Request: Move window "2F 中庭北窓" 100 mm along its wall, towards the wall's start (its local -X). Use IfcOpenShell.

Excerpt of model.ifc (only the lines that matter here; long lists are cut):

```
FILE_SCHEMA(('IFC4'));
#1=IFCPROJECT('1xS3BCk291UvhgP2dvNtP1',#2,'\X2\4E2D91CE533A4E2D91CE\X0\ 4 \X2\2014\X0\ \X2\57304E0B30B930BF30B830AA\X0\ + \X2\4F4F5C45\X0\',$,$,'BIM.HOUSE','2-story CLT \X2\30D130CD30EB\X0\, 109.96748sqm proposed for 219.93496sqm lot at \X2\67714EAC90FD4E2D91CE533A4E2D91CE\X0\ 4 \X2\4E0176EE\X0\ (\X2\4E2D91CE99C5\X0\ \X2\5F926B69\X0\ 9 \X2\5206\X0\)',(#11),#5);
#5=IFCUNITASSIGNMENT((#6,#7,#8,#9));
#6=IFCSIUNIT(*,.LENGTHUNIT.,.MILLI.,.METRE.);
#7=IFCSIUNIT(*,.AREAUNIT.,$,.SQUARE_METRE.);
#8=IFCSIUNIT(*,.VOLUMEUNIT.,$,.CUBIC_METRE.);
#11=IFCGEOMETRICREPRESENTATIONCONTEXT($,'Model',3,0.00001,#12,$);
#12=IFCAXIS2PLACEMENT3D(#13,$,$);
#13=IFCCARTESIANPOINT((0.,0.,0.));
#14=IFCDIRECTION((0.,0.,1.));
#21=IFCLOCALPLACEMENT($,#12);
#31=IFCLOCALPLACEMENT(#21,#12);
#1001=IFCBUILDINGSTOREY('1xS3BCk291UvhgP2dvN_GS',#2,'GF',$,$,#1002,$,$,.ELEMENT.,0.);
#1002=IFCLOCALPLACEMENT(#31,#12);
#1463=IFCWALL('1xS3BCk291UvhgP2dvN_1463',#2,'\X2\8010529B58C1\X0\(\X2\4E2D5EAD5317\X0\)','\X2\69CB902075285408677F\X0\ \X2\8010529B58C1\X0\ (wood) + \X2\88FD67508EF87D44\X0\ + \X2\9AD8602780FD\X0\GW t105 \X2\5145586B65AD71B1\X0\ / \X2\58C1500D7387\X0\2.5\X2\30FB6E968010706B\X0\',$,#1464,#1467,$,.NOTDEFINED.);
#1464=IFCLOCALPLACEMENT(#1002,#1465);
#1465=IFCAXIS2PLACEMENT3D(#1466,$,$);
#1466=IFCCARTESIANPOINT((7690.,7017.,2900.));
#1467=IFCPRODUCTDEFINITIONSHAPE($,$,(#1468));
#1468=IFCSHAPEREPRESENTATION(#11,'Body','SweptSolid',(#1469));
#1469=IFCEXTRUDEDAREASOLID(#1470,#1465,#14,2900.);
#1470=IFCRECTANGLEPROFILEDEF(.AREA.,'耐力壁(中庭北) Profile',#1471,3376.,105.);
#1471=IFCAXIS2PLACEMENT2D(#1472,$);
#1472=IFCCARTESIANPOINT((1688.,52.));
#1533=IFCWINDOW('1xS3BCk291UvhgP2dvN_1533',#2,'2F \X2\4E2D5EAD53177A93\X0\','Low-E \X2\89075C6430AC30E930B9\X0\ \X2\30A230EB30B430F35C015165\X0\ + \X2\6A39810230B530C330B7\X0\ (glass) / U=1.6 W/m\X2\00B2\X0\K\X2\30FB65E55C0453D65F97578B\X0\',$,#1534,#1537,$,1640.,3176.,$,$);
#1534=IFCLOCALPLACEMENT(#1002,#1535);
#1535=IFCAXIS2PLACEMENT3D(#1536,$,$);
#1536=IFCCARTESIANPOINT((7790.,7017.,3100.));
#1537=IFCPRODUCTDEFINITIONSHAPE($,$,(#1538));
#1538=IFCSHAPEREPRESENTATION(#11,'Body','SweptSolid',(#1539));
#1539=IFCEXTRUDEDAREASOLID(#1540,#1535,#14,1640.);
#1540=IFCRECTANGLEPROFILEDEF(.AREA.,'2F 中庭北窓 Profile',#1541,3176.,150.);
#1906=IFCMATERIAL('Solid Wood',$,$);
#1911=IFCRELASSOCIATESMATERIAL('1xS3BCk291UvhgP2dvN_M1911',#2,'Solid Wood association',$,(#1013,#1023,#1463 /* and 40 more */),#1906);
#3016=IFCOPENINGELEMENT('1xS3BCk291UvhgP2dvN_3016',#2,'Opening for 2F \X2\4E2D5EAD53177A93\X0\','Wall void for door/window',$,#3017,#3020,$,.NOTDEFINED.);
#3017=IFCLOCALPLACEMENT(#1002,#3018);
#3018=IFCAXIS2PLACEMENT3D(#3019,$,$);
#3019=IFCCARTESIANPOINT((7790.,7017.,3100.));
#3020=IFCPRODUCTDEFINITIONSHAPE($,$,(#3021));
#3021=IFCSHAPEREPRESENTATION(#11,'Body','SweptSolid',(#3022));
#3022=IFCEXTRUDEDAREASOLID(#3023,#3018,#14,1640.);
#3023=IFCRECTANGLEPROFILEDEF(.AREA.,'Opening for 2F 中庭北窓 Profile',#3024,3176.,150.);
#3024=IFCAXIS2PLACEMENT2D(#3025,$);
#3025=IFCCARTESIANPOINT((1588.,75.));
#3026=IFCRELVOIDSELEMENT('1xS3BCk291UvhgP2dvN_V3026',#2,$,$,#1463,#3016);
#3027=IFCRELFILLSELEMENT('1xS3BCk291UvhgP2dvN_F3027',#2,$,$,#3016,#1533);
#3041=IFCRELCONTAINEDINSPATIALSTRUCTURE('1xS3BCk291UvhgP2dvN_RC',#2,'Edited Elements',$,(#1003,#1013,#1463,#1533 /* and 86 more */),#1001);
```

```python
import ifcopenshell
import ifcopenshell.api.geometry
import ifcopenshell.util.placement
import ifcopenshell.util.unit

model = ifcopenshell.open("model.ifc")
unit_scale = ifcopenshell.util.unit.calculate_unit_scale(model)

window = model.by_guid("1xS3BCk291UvhgP2dvN_1533")
opening = window.FillsVoids[0].RelatingOpeningElement
wall = opening.VoidsElements[0].RelatingBuildingElement

wall_matrix = ifcopenshell.util.placement.get_local_placement(wall.ObjectPlacement)
shift = wall_matrix[:3, 0] * -0.1 / unit_scale
before = ifcopenshell.util.placement.get_local_placement(window.ObjectPlacement)[:3, 3].copy()

# The window is not placed relative to its opening, so move both.
for product in (opening, window):
    matrix = ifcopenshell.util.placement.get_local_placement(product.ObjectPlacement)
    matrix[:3, 3] += shift
    ifcopenshell.api.geometry.edit_object_placement(model, product=product, matrix=matrix, is_si=False)

after = ifcopenshell.util.placement.get_local_placement(window.ObjectPlacement)[:3, 3]
print("window moved by", (after - before).round(3) + 0.0)

model.write("model_v2.ifc")
```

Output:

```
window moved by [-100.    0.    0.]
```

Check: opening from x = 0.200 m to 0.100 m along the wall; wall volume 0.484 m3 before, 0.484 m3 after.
